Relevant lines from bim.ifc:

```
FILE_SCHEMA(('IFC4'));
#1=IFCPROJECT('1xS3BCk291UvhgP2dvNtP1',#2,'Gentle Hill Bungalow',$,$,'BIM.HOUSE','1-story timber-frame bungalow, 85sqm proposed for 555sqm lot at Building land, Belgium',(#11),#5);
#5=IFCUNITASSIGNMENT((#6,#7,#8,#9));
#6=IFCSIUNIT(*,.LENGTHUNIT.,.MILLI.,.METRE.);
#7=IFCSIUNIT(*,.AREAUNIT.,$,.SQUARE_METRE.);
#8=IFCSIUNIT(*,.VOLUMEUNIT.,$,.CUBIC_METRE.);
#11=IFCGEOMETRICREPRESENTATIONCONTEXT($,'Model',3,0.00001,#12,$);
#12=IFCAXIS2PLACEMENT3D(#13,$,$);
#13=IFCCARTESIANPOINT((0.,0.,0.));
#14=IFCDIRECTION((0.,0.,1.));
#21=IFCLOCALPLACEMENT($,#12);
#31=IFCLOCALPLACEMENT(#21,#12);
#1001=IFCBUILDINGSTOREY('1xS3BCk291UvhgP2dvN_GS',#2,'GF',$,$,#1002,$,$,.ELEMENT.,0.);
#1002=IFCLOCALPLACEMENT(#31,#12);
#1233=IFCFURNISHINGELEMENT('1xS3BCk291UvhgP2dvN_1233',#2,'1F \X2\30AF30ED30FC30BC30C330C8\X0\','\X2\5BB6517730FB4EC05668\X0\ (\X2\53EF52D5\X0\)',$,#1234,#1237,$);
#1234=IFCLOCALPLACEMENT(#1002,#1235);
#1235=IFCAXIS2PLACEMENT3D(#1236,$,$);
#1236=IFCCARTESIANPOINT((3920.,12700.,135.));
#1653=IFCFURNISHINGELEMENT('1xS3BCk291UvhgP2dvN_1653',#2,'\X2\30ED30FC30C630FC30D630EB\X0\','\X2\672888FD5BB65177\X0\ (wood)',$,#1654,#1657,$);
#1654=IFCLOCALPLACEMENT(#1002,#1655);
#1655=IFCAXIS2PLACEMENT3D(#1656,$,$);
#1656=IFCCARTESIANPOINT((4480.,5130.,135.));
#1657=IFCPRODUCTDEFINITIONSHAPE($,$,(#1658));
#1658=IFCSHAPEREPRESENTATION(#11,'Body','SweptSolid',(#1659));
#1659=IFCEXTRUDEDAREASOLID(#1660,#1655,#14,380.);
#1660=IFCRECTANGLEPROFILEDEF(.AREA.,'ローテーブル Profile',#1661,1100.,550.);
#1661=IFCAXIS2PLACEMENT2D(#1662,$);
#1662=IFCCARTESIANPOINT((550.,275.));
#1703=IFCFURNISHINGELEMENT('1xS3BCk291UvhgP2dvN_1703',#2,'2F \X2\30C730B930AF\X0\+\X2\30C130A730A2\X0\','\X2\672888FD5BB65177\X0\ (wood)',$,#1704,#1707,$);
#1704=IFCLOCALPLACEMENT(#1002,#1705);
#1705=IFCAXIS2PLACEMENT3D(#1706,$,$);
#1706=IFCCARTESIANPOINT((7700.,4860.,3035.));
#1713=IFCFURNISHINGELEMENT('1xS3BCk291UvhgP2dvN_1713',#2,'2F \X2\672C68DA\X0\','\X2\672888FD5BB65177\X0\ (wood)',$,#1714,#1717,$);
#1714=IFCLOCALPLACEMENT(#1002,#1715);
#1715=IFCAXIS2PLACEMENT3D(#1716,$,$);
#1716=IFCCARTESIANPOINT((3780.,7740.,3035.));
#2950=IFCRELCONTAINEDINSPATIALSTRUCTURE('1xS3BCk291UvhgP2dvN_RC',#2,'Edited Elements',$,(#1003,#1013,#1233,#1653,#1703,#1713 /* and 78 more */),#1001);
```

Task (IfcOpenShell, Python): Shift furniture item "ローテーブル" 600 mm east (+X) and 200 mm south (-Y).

```python
import ifcopenshell
import ifcopenshell.api.geometry
import ifcopenshell.util.placement

model = ifcopenshell.open("bim.ifc")

item = model.by_guid("1xS3BCk291UvhgP2dvN_1653")
matrix = ifcopenshell.util.placement.get_local_placement(item.ObjectPlacement)
matrix[0, 3] += 600.0
matrix[1, 3] -= 200.0
ifcopenshell.api.geometry.edit_object_placement(model, product=item, matrix=matrix, is_si=False)

print(ifcopenshell.util.placement.get_local_placement(item.ObjectPlacement).round(3) + 0.0)

model.write("bim_updated.ifc")
```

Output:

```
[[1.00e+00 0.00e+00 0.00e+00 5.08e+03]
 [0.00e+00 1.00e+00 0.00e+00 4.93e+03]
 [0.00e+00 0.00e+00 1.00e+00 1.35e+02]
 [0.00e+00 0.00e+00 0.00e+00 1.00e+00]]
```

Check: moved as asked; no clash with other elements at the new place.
